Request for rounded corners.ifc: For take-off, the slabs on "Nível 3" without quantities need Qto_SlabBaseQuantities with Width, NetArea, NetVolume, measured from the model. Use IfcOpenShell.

First a look at what the model holds.

```python
import ifcopenshell
import ifcopenshell.util.element
import ifcopenshell.util.unit

model = ifcopenshell.open("rounded corners.ifc")
print(model.schema)
for unit_type in ("LENGTHUNIT", "AREAUNIT", "VOLUMEUNIT"):
    print(unit_type, ifcopenshell.util.unit.calculate_unit_scale(model, unit_type))
storey = next(s for s in model.by_type("IfcBuildingStorey") if s.Name == "Nível 3")
slabs = [e for e in ifcopenshell.util.element.get_decomposition(storey) if e.is_a("IfcSlab")]
for e in sorted(slabs, key=lambda e: e.id()):
    print(e.id(), e.is_a(), e.Name, list(ifcopenshell.util.element.get_psets(e, qtos_only=True)), sep=" | ")
```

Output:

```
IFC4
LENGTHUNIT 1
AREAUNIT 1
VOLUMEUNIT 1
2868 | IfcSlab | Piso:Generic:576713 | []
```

```python
import ifcopenshell
import ifcopenshell.api.pset
import ifcopenshell.geom
import ifcopenshell.util.element
import ifcopenshell.util.shape
import ifcopenshell.util.unit

model = ifcopenshell.open("rounded corners.ifc")
unit_scale = ifcopenshell.util.unit.calculate_unit_scale(model)
area_scale = ifcopenshell.util.unit.calculate_unit_scale(model, "AREAUNIT")
volume_scale = ifcopenshell.util.unit.calculate_unit_scale(model, "VOLUMEUNIT")
settings = ifcopenshell.geom.settings()

storey = next(s for s in model.by_type("IfcBuildingStorey") if s.Name == "Nível 3")
slabs = [e for e in ifcopenshell.util.element.get_decomposition(storey) if e.is_a("IfcSlab")]

for e in sorted(slabs, key=lambda e: e.id()):
    if ifcopenshell.util.element.get_psets(e, qtos_only=True, should_inherit=False):
        continue
    # Geometry comes back in metres, in the element's own axes.
    shape = ifcopenshell.geom.create_shape(settings, e)
    values = {
        "Width": ifcopenshell.util.shape.get_z(shape.geometry) / unit_scale,
        "NetArea": ifcopenshell.util.shape.get_footprint_area(shape.geometry) / area_scale,
        "NetVolume": ifcopenshell.util.shape.get_volume(shape.geometry) / volume_scale,
    }
    qto = ifcopenshell.api.pset.add_qto(model, product=e, name="Qto_SlabBaseQuantities")
    ifcopenshell.api.pset.edit_qto(model, qto=qto, properties=values)
    print(e.id(), {k: round(v, 3) for k, v in values.items()})

model.write("rounded corners_rev.ifc")
```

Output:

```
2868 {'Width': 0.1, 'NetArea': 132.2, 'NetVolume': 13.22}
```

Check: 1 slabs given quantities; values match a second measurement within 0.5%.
